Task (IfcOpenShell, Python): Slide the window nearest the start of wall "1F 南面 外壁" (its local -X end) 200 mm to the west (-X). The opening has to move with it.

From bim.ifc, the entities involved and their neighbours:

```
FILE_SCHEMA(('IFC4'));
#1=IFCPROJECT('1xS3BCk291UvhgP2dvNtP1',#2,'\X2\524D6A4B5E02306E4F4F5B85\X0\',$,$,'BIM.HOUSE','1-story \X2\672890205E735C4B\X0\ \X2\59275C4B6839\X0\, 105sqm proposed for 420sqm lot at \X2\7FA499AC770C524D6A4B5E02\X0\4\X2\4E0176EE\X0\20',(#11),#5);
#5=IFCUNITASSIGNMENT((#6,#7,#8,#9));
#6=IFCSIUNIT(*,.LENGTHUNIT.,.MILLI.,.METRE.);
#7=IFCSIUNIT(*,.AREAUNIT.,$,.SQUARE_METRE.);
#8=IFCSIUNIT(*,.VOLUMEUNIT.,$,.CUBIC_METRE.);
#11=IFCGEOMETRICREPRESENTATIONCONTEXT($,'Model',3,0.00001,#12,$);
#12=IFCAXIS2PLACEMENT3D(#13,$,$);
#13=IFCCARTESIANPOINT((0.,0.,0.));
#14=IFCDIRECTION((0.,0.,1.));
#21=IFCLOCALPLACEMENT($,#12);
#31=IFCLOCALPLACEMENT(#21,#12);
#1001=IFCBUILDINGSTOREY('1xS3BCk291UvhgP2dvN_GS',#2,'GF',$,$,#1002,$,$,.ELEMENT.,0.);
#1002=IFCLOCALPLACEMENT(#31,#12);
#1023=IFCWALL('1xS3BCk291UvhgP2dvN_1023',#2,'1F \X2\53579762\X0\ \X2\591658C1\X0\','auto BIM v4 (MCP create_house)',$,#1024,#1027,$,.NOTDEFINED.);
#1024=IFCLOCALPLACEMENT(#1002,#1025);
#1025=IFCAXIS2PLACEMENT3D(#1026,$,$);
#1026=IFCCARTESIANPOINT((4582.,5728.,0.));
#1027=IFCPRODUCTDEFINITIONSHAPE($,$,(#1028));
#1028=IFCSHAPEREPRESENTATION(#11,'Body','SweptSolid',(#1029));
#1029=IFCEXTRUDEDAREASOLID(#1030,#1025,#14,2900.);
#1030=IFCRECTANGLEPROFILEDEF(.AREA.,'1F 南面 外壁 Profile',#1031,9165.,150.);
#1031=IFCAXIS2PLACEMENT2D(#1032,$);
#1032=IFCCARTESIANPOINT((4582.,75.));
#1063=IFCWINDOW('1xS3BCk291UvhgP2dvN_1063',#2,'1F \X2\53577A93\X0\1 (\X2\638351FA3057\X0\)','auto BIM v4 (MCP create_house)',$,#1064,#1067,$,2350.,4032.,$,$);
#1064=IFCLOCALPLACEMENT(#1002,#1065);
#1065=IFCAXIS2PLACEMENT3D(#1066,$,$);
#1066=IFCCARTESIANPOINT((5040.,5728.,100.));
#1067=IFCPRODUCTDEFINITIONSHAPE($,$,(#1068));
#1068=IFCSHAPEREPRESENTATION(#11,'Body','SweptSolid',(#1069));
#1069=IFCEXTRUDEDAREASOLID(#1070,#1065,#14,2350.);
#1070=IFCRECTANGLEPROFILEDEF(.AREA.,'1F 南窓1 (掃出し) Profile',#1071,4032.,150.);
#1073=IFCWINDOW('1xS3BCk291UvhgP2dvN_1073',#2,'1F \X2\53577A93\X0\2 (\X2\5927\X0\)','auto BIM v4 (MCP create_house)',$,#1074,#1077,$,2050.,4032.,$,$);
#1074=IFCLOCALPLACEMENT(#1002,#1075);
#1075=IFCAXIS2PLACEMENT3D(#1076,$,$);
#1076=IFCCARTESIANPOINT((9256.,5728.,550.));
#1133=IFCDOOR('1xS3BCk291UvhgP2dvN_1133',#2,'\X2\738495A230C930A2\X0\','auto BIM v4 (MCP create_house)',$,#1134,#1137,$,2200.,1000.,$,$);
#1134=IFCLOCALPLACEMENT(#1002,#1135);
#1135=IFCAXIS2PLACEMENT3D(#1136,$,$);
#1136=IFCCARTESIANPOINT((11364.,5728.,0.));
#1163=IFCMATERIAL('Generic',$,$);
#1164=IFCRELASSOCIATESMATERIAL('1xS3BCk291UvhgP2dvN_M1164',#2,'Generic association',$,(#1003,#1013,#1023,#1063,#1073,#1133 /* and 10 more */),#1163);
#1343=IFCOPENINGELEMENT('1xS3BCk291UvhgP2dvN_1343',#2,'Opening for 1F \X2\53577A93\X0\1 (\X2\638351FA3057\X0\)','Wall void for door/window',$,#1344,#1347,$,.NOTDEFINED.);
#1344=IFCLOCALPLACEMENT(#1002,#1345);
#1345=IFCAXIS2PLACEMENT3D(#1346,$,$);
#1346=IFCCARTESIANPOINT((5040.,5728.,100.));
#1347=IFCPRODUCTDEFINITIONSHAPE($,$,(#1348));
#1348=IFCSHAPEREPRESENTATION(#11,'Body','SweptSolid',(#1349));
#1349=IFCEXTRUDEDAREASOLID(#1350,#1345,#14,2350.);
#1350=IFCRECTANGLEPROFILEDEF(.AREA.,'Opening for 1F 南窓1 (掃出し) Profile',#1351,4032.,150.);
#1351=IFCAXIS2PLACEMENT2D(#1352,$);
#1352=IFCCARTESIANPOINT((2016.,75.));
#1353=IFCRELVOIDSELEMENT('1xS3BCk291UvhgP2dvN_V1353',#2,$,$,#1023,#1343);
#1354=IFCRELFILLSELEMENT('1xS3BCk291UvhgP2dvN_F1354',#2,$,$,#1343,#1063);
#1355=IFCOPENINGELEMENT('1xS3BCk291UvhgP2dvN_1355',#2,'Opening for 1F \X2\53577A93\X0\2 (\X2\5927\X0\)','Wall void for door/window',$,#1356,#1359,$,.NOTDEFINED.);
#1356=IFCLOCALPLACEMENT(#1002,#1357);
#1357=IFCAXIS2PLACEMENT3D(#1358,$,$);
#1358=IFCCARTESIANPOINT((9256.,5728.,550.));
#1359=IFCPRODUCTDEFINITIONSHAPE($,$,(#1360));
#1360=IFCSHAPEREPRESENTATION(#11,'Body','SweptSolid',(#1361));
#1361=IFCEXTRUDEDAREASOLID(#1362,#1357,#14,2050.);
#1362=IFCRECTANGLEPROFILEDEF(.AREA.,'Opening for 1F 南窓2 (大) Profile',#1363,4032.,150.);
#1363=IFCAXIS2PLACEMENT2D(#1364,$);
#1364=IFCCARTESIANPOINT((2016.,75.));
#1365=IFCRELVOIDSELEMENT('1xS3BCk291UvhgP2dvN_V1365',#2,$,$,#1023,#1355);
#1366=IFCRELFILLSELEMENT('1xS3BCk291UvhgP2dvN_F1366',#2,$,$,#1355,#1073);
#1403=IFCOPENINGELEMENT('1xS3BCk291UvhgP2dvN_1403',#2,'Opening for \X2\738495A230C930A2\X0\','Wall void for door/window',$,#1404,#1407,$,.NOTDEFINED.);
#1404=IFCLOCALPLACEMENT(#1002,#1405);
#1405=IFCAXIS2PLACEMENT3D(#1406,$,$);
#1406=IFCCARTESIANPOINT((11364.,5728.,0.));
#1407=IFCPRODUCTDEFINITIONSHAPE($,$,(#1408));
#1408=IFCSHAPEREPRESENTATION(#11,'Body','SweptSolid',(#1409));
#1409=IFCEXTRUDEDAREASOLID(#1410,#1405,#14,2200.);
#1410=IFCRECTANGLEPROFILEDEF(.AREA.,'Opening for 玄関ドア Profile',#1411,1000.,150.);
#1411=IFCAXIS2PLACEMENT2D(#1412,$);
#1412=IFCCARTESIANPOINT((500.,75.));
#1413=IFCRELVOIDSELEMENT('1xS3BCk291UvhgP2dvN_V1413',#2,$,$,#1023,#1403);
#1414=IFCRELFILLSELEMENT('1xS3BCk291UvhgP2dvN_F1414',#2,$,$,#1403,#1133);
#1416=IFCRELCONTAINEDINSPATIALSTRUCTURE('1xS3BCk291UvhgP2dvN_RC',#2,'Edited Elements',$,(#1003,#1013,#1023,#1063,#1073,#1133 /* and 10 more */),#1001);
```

```python
import ifcopenshell
import ifcopenshell.api.geometry
import ifcopenshell.util.placement
import ifcopenshell.util.unit

model = ifcopenshell.open("bim.ifc")
unit_scale = ifcopenshell.util.unit.calculate_unit_scale(model)

window = model.by_guid("1xS3BCk291UvhgP2dvN_1063")
opening = window.FillsVoids[0].RelatingOpeningElement
wall = opening.VoidsElements[0].RelatingBuildingElement

wall_matrix = ifcopenshell.util.placement.get_local_placement(wall.ObjectPlacement)
shift = wall_matrix[:3, 0] * -0.2 / unit_scale
before = ifcopenshell.util.placement.get_local_placement(window.ObjectPlacement)[:3, 3].copy()

# The window is not placed relative to its opening, so move both.
for product in (opening, window):
    matrix = ifcopenshell.util.placement.get_local_placement(product.ObjectPlacement)
    matrix[:3, 3] += shift
    ifcopenshell.api.geometry.edit_object_placement(model, product=product, matrix=matrix, is_si=False)

after = ifcopenshell.util.placement.get_local_placement(window.ObjectPlacement)[:3, 3]
print("window moved by", (after - before).round(3) + 0.0)

model.write("bim-out.ifc")
```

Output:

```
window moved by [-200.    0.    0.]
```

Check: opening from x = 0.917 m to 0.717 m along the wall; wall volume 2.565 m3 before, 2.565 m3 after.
